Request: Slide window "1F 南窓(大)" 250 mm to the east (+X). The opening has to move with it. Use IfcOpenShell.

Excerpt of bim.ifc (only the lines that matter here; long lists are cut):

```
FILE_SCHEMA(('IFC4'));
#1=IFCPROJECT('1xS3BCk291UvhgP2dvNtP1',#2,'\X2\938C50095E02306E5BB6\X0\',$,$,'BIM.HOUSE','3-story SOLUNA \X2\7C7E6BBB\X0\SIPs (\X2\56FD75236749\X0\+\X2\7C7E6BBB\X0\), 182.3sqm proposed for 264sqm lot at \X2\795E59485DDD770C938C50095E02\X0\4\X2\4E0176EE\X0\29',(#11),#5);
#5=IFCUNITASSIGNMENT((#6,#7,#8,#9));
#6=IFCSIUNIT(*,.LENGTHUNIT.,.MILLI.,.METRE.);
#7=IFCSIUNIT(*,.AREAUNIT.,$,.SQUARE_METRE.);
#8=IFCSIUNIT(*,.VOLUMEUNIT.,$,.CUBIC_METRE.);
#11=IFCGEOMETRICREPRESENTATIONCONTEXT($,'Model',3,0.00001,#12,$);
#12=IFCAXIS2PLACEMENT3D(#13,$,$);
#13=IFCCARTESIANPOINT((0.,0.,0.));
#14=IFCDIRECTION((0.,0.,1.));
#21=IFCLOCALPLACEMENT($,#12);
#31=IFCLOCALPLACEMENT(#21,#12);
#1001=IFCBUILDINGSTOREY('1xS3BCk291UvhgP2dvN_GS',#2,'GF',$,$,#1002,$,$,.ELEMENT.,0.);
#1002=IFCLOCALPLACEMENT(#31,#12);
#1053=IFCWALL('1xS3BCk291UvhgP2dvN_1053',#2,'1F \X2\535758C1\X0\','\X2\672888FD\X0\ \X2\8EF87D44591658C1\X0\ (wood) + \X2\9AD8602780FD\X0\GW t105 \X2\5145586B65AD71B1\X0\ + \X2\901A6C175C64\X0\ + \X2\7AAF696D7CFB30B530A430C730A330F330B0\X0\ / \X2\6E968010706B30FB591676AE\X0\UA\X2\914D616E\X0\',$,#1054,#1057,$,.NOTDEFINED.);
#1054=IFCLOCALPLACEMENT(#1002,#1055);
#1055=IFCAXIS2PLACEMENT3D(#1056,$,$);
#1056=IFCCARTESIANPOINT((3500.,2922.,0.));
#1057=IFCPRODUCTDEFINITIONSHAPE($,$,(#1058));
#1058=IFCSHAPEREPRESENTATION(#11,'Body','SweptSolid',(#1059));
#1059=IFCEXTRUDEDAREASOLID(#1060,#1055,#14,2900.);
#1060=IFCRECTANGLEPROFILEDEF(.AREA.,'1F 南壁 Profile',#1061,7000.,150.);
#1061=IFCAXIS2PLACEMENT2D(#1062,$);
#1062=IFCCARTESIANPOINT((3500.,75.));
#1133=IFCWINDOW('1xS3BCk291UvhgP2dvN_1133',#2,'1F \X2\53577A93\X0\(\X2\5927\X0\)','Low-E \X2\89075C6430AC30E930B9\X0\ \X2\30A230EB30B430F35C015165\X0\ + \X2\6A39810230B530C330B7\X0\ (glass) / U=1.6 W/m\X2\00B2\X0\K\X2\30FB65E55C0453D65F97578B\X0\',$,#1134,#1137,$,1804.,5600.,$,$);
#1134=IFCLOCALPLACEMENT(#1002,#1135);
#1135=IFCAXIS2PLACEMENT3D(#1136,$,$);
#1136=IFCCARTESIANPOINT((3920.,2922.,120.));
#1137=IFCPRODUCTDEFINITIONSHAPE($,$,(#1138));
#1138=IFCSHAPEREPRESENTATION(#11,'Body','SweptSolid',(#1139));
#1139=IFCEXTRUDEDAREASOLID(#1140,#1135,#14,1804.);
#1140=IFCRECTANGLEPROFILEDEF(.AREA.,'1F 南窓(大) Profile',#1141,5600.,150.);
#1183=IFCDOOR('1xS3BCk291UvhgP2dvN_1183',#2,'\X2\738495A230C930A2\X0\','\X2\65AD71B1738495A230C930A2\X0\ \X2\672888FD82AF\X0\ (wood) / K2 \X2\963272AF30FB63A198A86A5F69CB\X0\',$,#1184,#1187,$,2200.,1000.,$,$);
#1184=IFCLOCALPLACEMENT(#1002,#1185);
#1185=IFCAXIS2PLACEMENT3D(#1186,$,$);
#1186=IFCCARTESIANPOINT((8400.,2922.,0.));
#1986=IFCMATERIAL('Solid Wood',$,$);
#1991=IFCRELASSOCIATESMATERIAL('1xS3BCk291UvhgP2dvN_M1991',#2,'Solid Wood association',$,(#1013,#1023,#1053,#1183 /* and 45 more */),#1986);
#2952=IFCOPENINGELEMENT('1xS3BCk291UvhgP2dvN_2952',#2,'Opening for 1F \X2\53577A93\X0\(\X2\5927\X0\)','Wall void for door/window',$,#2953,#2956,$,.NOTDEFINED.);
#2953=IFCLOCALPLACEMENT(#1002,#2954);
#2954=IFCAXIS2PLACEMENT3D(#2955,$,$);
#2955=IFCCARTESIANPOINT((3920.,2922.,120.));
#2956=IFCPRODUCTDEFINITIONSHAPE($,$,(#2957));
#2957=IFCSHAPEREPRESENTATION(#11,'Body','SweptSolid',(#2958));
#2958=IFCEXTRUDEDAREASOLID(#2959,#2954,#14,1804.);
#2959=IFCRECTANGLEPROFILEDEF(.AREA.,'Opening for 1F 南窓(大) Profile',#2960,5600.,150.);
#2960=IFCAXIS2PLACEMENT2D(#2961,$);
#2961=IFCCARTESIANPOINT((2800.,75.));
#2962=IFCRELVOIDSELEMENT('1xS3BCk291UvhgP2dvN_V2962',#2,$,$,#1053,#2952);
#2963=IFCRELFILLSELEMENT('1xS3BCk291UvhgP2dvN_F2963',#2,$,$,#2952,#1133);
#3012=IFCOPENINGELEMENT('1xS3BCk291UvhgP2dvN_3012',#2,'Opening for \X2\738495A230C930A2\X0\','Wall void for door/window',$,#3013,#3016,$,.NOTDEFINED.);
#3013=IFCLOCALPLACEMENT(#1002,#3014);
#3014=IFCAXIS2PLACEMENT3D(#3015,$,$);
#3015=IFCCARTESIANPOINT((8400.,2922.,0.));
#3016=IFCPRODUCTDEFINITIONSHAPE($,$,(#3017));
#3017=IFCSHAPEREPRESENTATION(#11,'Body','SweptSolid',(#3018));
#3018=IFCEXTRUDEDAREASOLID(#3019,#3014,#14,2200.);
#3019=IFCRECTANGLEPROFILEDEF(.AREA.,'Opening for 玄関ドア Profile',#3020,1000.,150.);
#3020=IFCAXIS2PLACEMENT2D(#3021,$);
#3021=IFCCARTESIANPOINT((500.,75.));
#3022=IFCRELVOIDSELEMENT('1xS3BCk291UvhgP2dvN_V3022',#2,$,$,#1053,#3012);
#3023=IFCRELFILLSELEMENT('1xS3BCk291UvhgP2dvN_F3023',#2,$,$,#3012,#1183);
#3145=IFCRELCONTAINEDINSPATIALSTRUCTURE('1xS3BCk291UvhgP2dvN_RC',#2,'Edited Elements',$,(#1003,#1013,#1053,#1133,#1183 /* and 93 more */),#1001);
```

```python
import ifcopenshell
import ifcopenshell.api.geometry
import ifcopenshell.util.placement

model = ifcopenshell.open("bim.ifc")

window = model.by_id(1133)
opening = window.FillsVoids[0].RelatingOpeningElement
wall = opening.VoidsElements[0].RelatingBuildingElement

wall_matrix = ifcopenshell.util.placement.get_local_placement(wall.ObjectPlacement)
shift = wall_matrix[:3, 0] * 250.0
before = ifcopenshell.util.placement.get_local_placement(window.ObjectPlacement)[:3, 3].copy()

# The window is not placed relative to its opening, so move both.
for product in (opening, window):
    matrix = ifcopenshell.util.placement.get_local_placement(product.ObjectPlacement)
    matrix[:3, 3] += shift
    ifcopenshell.api.geometry.edit_object_placement(model, product=product, matrix=matrix, is_si=False)

after = ifcopenshell.util.placement.get_local_placement(window.ObjectPlacement)[:3, 3]
print("window moved by", (after - before).round(3) + 0.0)

model.write("bim_updated.ifc")
```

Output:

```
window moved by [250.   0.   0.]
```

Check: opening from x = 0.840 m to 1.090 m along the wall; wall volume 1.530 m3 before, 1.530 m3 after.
